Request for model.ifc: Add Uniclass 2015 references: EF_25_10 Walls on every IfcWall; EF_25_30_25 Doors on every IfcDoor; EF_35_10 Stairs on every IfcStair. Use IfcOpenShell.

First a look at what the model holds.

```python
import ifcopenshell

model = ifcopenshell.open("model.ifc")
print(model.schema)
print("classifications:", [c.Name for c in model.by_type("IfcClassification")])
for ifc_class in ("IfcDoor", "IfcRoof", "IfcStair", "IfcWall", "IfcWindow"):
    print(ifc_class, len(model.by_type(ifc_class)))
```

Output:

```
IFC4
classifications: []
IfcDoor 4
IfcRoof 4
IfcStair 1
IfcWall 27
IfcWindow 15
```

```python
import ifcopenshell
import ifcopenshell.api.classification

model = ifcopenshell.open("model.ifc")

system = ifcopenshell.api.classification.add_classification(model, classification="Uniclass 2015")

codes = {
    "IfcWall": ("EF_25_10", "Walls"),
    "IfcDoor": ("EF_25_30_25", "Doors"),
    "IfcStair": ("EF_35_10", "Stairs"),
}
for ifc_class, (code, name) in codes.items():
    products = model.by_type(ifc_class)
    ifcopenshell.api.classification.add_reference(
        model, products=products, classification=system, identification=code, name=name
    )
    print(code, len(products))

model.write("model_v2.ifc")
```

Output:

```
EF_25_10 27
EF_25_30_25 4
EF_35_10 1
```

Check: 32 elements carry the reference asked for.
